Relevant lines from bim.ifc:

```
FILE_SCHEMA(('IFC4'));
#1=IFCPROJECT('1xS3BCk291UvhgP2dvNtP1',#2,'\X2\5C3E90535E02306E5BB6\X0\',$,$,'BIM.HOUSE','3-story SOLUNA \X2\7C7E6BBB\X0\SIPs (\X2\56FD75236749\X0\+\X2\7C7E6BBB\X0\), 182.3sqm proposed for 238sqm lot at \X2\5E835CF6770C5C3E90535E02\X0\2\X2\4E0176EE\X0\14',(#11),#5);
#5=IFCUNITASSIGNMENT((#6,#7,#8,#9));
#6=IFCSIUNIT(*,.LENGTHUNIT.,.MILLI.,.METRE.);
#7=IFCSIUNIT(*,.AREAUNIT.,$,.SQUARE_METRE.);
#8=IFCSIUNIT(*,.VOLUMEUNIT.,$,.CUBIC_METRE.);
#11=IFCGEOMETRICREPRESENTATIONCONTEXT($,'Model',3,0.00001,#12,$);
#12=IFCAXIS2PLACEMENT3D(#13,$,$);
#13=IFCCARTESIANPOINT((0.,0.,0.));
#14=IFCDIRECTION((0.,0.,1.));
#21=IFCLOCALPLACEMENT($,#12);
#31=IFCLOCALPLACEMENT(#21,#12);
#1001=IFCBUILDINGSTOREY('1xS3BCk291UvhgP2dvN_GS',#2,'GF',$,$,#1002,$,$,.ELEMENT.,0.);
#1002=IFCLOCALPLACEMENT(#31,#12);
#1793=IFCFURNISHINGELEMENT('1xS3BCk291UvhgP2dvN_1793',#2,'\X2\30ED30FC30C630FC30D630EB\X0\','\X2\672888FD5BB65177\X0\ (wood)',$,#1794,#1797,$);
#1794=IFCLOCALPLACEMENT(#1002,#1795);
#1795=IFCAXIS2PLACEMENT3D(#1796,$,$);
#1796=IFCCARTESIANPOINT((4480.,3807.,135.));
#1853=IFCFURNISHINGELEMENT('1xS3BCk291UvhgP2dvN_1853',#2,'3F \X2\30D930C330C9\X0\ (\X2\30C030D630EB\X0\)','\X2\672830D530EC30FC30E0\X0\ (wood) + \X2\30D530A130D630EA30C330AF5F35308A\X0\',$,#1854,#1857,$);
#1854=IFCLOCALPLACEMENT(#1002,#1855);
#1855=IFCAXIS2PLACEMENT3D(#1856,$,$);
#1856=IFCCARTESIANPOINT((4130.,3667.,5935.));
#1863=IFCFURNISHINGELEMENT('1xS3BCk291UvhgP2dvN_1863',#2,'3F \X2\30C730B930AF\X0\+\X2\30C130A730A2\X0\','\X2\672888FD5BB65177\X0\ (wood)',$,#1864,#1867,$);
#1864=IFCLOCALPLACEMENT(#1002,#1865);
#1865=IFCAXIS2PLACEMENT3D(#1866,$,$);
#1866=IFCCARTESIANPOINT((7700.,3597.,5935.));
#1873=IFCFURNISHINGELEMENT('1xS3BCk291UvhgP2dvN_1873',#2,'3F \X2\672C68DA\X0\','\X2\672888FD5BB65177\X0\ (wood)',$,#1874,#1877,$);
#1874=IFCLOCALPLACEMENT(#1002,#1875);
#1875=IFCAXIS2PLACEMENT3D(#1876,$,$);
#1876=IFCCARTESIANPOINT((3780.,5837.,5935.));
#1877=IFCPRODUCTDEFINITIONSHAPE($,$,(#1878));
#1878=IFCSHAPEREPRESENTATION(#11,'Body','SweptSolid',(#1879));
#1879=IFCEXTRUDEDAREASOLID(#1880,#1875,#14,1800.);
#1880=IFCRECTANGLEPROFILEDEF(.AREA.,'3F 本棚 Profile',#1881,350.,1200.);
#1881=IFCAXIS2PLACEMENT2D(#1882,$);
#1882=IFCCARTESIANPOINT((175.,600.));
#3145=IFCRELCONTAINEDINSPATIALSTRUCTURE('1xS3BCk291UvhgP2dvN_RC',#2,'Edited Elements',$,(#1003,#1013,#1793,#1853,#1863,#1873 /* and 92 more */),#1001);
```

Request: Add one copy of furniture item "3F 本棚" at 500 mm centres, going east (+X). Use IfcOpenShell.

```python
import numpy as np
import ifcopenshell
import ifcopenshell.api.geometry
import ifcopenshell.api.root
import ifcopenshell.util.element
import ifcopenshell.util.placement
import ifcopenshell.util.unit

model = ifcopenshell.open("bim.ifc")
unit_scale = ifcopenshell.util.unit.calculate_unit_scale(model)


def reuse_history(source, copy):
    """copy_class also copies each property set's owner history, people and application; keep the originals."""
    for rel in copy.IsDefinedBy:
        if rel.is_a("IfcRelDefinesByProperties") and (history := rel.RelatingPropertyDefinition.OwnerHistory):
            rel.RelatingPropertyDefinition.OwnerHistory = source.OwnerHistory
            ifcopenshell.util.element.remove_deep2(model, history)


source = model.by_guid("1xS3BCk291UvhgP2dvN_1873")
base = ifcopenshell.util.placement.get_local_placement(source.ObjectPlacement)
step = np.array([1.0, 0.0, 0.0]) * 0.5 / unit_scale

for i in range(1, 2):
    copy = ifcopenshell.api.root.copy_class(model, product=source)
    copy.Representation = ifcopenshell.util.element.copy_deep(
        model, source.Representation, exclude=["IfcGeometricRepresentationContext", "IfcRepresentationMap"]
    )
    reuse_history(source, copy)
    matrix = base.copy()
    matrix[:3, 3] += i * step
    print("added at", matrix[:3, 3].round(3) + 0.0)
    ifcopenshell.api.geometry.edit_object_placement(model, product=copy, matrix=matrix, is_si=False)

model.write("bim_v2.ifc")
```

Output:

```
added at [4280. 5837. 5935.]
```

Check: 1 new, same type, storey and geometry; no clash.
